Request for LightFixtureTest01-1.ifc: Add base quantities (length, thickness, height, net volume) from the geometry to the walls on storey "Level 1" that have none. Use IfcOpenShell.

First a look at what the model holds.

```python
import ifcopenshell
import ifcopenshell.util.element
import ifcopenshell.util.unit

model = ifcopenshell.open("LightFixtureTest01-1.ifc")
print(model.schema)
for unit_type in ("LENGTHUNIT", "AREAUNIT", "VOLUMEUNIT"):
    print(unit_type, ifcopenshell.util.unit.calculate_unit_scale(model, unit_type))
storey = next(s for s in model.by_type("IfcBuildingStorey") if s.Name == "Level 1")
walls = [e for e in ifcopenshell.util.element.get_decomposition(storey) if e.is_a("IfcWall")]
for e in sorted(walls, key=lambda e: e.id()):
    print(e.id(), e.is_a(), e.Name, list(ifcopenshell.util.element.get_psets(e, qtos_only=True)), sep=" | ")
```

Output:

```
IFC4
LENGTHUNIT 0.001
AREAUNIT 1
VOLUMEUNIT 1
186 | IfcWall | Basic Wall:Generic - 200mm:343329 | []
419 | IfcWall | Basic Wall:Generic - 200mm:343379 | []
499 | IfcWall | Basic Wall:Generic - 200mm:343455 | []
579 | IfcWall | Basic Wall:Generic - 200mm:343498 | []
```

```python
import ifcopenshell
import ifcopenshell.api.pset
import ifcopenshell.geom
import ifcopenshell.util.element
import ifcopenshell.util.shape
import ifcopenshell.util.unit

model = ifcopenshell.open("LightFixtureTest01-1.ifc")
unit_scale = ifcopenshell.util.unit.calculate_unit_scale(model)
volume_scale = ifcopenshell.util.unit.calculate_unit_scale(model, "VOLUMEUNIT")
settings = ifcopenshell.geom.settings()

storey = next(s for s in model.by_type("IfcBuildingStorey") if s.Name == "Level 1")
walls = [e for e in ifcopenshell.util.element.get_decomposition(storey) if e.is_a("IfcWall")]

for e in sorted(walls, key=lambda e: e.id()):
    if ifcopenshell.util.element.get_psets(e, qtos_only=True, should_inherit=False):
        continue
    # Geometry comes back in metres, in the element's own axes.
    shape = ifcopenshell.geom.create_shape(settings, e)
    values = {
        "Length": ifcopenshell.util.shape.get_x(shape.geometry) / unit_scale,
        "Width": ifcopenshell.util.shape.get_y(shape.geometry) / unit_scale,
        "Height": ifcopenshell.util.shape.get_z(shape.geometry) / unit_scale,
        "NetVolume": ifcopenshell.util.shape.get_volume(shape.geometry) / volume_scale,
    }
    qto = ifcopenshell.api.pset.add_qto(model, product=e, name="Qto_WallBaseQuantities")
    ifcopenshell.api.pset.edit_qto(model, qto=qto, properties=values)
    print(e.id(), {k: round(v, 3) for k, v in values.items()})

model.write("LightFixtureTest01-1_v2.ifc")
```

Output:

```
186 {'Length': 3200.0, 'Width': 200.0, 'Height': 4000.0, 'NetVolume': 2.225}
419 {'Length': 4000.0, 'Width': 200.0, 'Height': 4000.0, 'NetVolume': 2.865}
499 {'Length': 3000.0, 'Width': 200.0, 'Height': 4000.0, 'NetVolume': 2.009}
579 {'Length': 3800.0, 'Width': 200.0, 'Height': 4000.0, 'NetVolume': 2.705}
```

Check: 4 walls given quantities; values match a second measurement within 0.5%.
